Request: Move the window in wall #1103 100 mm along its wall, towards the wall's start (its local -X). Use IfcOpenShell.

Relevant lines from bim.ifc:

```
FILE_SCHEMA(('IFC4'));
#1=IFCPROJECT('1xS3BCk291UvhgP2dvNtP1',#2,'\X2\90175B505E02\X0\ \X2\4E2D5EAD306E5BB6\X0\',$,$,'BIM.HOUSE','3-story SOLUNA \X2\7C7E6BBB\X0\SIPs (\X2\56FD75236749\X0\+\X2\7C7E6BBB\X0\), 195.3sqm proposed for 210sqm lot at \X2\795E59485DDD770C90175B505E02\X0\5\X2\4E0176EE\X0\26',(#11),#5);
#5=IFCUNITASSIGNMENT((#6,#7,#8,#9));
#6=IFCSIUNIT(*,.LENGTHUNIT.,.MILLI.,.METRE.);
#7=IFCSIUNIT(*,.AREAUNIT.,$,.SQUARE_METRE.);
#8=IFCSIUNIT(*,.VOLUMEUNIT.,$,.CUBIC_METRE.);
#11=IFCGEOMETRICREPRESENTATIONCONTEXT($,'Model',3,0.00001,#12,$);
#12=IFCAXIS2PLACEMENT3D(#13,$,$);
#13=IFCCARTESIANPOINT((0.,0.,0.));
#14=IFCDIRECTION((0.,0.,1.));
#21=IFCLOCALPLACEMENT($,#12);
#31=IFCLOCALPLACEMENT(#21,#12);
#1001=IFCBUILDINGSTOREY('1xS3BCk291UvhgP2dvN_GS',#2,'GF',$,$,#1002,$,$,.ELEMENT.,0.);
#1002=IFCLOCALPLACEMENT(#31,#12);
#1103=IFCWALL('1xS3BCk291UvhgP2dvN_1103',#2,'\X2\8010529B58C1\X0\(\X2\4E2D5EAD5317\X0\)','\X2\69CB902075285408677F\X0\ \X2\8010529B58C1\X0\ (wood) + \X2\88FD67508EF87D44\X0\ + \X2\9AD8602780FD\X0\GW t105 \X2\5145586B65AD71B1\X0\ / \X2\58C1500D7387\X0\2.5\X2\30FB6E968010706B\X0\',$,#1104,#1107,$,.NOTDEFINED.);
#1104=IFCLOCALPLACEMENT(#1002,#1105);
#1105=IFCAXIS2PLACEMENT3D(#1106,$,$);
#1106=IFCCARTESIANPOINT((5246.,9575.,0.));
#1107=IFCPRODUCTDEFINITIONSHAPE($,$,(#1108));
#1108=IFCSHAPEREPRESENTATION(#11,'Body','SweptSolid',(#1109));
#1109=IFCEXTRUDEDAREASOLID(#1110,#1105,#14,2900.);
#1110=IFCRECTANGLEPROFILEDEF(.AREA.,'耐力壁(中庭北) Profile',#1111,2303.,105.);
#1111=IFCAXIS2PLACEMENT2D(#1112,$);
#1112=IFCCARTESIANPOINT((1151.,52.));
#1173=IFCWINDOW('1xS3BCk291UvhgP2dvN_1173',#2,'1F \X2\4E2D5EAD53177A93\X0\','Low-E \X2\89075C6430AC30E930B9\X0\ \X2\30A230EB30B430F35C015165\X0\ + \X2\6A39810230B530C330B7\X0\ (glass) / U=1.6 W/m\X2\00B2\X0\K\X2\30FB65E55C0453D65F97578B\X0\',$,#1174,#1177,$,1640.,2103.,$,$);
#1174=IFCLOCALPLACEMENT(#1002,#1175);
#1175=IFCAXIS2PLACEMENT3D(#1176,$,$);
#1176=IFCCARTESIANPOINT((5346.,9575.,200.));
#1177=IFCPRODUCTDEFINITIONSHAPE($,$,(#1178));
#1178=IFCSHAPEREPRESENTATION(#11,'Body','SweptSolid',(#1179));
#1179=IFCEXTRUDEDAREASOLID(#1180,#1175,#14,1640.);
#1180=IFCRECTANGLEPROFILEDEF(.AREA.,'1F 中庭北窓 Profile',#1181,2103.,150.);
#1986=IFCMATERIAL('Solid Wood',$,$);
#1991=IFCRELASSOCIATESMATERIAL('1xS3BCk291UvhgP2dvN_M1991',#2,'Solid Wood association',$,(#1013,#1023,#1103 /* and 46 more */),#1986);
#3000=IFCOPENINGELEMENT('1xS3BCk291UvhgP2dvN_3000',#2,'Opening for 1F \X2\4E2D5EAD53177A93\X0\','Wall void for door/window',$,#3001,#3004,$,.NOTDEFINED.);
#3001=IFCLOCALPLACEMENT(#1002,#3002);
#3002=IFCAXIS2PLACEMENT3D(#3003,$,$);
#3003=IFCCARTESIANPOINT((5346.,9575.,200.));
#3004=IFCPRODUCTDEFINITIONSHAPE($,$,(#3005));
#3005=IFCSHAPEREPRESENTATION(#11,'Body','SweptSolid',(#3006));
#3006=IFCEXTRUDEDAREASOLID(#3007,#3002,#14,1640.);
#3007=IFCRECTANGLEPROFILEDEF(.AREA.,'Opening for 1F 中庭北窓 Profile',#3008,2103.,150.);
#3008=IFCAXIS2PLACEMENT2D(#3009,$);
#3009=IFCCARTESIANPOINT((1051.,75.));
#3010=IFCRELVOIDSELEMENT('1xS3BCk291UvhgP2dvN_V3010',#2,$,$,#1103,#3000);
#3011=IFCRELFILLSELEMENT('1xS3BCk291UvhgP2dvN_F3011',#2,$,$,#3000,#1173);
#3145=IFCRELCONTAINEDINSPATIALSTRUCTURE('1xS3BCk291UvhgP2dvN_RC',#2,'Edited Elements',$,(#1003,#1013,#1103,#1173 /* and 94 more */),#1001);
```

```python
import ifcopenshell
import ifcopenshell.api.geometry
import ifcopenshell.util.placement

model = ifcopenshell.open("bim.ifc")

window = model.by_guid("1xS3BCk291UvhgP2dvN_1173")
opening = window.FillsVoids[0].RelatingOpeningElement
wall = opening.VoidsElements[0].RelatingBuildingElement

wall_matrix = ifcopenshell.util.placement.get_local_placement(wall.ObjectPlacement)
shift = wall_matrix[:3, 0] * -100.0
before = ifcopenshell.util.placement.get_local_placement(window.ObjectPlacement)[:3, 3].copy()

# The window is not placed relative to its opening, so move both.
for product in (opening, window):
    matrix = ifcopenshell.util.placement.get_local_placement(product.ObjectPlacement)
    matrix[:3, 3] += shift
    ifcopenshell.api.geometry.edit_object_placement(model, product=product, matrix=matrix, is_si=False)

after = ifcopenshell.util.placement.get_local_placement(window.ObjectPlacement)[:3, 3]
print("window moved by", (after - before).round(3) + 0.0)

model.write("bim_updated.ifc")
```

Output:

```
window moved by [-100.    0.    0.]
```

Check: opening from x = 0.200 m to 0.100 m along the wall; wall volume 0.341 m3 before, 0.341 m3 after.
